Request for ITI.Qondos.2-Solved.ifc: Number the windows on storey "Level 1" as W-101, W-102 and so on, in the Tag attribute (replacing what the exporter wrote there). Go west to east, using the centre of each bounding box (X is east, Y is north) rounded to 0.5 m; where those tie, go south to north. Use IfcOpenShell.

First a look at what the model holds.

```python
import ifcopenshell
import ifcopenshell.util.element
import ifcopenshell.util.placement

model = ifcopenshell.open("ITI.Qondos.2-Solved.ifc")
print(model.schema)
storey = next(s for s in model.by_type("IfcBuildingStorey") if s.Name == "Level 1")
windows = [e for e in ifcopenshell.util.element.get_decomposition(storey) if e.is_a("IfcWindow")]
for e in sorted(windows, key=lambda e: e.id()):
    origin = ifcopenshell.util.placement.get_local_placement(e.ObjectPlacement)[:3, 3]
    print(e.id(), e.Tag, e.Name, origin.round(2) + 0.0, sep=" | ")
```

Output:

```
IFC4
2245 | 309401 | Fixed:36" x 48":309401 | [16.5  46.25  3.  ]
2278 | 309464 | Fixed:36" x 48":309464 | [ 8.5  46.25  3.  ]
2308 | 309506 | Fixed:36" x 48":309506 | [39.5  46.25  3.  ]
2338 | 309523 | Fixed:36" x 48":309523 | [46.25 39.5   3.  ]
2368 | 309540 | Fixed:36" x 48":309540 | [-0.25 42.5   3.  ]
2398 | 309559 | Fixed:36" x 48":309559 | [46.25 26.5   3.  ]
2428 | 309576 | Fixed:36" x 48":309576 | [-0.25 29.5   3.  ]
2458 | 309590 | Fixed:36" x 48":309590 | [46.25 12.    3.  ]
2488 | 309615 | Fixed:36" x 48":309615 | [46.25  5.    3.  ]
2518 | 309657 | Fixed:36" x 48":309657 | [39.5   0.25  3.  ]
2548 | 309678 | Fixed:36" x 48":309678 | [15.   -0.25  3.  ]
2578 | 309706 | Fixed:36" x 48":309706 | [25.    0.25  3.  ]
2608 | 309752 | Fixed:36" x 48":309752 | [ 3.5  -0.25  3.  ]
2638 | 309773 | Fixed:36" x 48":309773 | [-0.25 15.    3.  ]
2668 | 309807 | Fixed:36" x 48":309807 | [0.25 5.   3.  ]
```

```python
import ifcopenshell
import ifcopenshell.geom
import ifcopenshell.util.element
import ifcopenshell.util.shape

model = ifcopenshell.open("ITI.Qondos.2-Solved.ifc")
settings = ifcopenshell.geom.settings()
settings.set("use-world-coords", True)


def centre(element):
    shape = ifcopenshell.geom.create_shape(settings, element)
    return ifcopenshell.util.shape.get_bbox_centroid(shape.geometry)


storey = next(s for s in model.by_type("IfcBuildingStorey") if s.Name == "Level 1")
windows = [e for e in ifcopenshell.util.element.get_decomposition(storey) if e.is_a("IfcWindow")]

# Insertion points can sit at a corner or the storey origin, so sort by the geometry (in metres).
centres = {e: centre(e) for e in windows}
windows.sort(key=lambda e: (round(centres[e][0] / 0.5), centres[e][1]))

for i, e in enumerate(windows, start=1):
    number = f"W-1{i:02d}"
    e.Tag = number
    print(e.id(), number)

model.write("ITI.Qondos.2-Solved_v2.ifc")
```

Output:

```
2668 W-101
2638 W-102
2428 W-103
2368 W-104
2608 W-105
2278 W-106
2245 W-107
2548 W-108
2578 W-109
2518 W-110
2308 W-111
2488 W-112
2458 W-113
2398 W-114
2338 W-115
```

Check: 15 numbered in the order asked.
